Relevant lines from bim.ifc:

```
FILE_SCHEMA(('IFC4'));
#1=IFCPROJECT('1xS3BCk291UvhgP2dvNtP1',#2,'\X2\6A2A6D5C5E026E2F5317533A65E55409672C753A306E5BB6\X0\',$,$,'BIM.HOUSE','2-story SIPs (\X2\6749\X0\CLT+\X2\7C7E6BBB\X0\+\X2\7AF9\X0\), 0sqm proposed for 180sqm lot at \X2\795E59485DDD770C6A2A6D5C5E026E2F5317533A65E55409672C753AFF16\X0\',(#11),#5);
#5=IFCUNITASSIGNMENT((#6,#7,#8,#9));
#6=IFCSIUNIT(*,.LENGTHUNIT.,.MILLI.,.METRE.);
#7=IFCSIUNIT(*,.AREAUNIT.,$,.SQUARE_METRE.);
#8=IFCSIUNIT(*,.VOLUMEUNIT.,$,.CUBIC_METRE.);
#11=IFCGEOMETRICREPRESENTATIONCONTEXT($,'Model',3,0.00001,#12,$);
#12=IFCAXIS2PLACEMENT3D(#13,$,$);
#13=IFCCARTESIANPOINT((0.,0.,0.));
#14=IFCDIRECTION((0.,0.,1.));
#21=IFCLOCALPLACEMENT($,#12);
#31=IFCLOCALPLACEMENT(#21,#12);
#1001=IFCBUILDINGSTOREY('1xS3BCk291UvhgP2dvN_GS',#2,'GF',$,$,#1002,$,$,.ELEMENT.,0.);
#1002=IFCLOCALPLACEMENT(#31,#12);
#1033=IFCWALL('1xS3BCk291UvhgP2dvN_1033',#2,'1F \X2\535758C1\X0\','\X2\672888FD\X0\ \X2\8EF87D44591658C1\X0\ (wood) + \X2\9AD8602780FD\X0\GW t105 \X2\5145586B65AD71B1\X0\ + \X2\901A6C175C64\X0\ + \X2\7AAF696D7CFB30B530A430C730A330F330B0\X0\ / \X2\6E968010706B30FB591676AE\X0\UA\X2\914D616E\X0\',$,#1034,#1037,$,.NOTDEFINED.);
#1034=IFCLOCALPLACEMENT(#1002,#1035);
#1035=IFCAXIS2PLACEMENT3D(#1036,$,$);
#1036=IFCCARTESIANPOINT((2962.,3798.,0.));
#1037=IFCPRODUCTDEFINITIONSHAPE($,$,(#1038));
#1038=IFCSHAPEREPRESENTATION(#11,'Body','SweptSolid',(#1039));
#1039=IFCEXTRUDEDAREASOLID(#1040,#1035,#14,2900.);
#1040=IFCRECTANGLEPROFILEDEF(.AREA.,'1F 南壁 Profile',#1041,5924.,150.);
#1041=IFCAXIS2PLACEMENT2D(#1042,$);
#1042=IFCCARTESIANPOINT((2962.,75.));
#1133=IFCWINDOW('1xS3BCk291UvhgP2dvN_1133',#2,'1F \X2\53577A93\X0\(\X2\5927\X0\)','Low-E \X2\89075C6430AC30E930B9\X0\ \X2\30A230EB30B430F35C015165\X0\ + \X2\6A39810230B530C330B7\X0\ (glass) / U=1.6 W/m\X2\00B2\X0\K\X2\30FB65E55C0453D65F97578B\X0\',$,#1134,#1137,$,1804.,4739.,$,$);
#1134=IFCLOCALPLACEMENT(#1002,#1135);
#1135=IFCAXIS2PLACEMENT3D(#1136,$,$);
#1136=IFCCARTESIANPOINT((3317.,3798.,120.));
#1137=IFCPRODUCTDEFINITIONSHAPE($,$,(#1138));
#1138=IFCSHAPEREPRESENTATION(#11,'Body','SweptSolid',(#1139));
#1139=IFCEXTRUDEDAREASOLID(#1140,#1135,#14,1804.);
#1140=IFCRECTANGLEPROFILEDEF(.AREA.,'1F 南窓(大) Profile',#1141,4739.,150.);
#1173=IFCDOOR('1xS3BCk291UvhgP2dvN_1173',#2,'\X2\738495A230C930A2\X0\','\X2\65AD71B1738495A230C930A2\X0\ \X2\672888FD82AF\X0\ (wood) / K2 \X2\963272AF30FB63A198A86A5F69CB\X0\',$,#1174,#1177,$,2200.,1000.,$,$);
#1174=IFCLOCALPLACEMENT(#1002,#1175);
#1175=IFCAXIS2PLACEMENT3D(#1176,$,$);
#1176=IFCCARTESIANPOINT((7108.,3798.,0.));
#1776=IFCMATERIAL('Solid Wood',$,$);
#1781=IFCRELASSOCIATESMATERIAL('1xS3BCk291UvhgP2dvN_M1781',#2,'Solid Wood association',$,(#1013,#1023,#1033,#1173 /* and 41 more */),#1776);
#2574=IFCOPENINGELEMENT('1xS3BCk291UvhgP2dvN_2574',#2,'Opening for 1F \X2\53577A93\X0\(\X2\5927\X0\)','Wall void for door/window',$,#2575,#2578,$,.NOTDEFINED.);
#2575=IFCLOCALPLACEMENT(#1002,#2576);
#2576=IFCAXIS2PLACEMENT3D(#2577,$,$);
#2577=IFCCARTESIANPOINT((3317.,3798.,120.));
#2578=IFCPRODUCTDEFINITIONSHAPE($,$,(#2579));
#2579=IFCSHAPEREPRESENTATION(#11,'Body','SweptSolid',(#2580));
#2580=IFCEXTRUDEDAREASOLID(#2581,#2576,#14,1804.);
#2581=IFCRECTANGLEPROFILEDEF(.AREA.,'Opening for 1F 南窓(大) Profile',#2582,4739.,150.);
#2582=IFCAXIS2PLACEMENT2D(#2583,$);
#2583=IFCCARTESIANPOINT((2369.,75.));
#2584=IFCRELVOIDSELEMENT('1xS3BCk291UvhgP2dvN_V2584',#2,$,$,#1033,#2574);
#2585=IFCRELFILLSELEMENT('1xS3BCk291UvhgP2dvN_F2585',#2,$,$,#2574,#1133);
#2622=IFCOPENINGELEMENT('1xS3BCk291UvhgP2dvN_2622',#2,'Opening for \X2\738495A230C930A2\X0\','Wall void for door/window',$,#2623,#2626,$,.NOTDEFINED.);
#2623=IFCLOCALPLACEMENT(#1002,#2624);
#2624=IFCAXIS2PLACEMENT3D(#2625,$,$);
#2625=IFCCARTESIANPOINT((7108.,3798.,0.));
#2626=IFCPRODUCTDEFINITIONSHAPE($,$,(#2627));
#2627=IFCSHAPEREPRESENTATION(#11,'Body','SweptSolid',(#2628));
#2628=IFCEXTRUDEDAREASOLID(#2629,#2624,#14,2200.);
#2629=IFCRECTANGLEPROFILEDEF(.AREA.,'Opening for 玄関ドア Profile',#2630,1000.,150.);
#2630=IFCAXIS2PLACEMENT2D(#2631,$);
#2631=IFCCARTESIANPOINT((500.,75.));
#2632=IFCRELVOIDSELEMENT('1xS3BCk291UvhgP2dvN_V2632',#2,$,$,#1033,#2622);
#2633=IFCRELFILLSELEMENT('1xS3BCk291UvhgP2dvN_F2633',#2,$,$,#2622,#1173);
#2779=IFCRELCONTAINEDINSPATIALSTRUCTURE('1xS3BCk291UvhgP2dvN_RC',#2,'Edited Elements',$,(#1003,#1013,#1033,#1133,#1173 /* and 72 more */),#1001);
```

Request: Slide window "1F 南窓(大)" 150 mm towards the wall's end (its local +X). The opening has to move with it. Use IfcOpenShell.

```python
import ifcopenshell
import ifcopenshell.api.geometry
import ifcopenshell.util.placement
import ifcopenshell.util.unit

model = ifcopenshell.open("bim.ifc")
unit_scale = ifcopenshell.util.unit.calculate_unit_scale(model)

window = model.by_guid("1xS3BCk291UvhgP2dvN_1133")
opening = window.FillsVoids[0].RelatingOpeningElement
wall = opening.VoidsElements[0].RelatingBuildingElement

wall_matrix = ifcopenshell.util.placement.get_local_placement(wall.ObjectPlacement)
shift = wall_matrix[:3, 0] * 0.15 / unit_scale
before = ifcopenshell.util.placement.get_local_placement(window.ObjectPlacement)[:3, 3].copy()

# The window is not placed relative to its opening, so move both.
for product in (opening, window):
    matrix = ifcopenshell.util.placement.get_local_placement(product.ObjectPlacement)
    matrix[:3, 3] += shift
    ifcopenshell.api.geometry.edit_object_placement(model, product=product, matrix=matrix, is_si=False)

after = ifcopenshell.util.placement.get_local_placement(window.ObjectPlacement)[:3, 3]
print("window moved by", (after - before).round(3) + 0.0)

model.write("bim_v2.ifc")
```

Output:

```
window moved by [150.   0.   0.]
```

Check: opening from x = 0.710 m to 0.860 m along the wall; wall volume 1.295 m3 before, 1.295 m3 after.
